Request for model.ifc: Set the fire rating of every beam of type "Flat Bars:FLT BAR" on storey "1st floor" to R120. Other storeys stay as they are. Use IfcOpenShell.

First a look at what the model holds.

```python
import ifcopenshell
import ifcopenshell.util.element

model = ifcopenshell.open("model.ifc")
print(model.schema)
storey = next(s for s in model.by_type("IfcBuildingStorey") if s.Name == "1st floor")
beams = [e for e in ifcopenshell.util.element.get_decomposition(storey) if e.is_a("IfcBeam")]
seen = {}
for e in beams:
    element_type = ifcopenshell.util.element.get_type(e)
    key = (element_type.Name if element_type != e and element_type else None, ifcopenshell.util.element.get_pset(e, "Pset_BeamCommon", "FireRating"))
    seen[key] = seen.get(key, 0) + 1
for (name, value), count in sorted(seen.items(), key=str):
    print(count, "x", name, "|", value)
```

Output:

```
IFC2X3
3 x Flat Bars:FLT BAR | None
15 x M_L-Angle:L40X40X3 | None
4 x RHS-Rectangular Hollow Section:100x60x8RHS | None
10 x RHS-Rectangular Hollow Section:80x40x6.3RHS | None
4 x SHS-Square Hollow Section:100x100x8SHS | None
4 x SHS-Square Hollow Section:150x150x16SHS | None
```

```python
import ifcopenshell
import ifcopenshell.api.pset
import ifcopenshell.util.element

model = ifcopenshell.open("model.ifc")

storey = next(s for s in model.by_type("IfcBuildingStorey") if s.Name == "1st floor")
beams = [e for e in ifcopenshell.util.element.get_decomposition(storey) if e.is_a("IfcBeam")]

count = 0
for e in beams:
    element_type = ifcopenshell.util.element.get_type(e)
    if element_type in (None, e) or element_type.Name != "Flat Bars:FLT BAR":
        continue
    # add_pset returns the element's existing set when there is one.
    pset = ifcopenshell.api.pset.add_pset(model, product=e, name="Pset_BeamCommon")
    ifcopenshell.api.pset.edit_pset(model, pset=pset, properties={"FireRating": "R120"})
    count += 1

print(count, "beams updated")

model.write("model-out.ifc")
```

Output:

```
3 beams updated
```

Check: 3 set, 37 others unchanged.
